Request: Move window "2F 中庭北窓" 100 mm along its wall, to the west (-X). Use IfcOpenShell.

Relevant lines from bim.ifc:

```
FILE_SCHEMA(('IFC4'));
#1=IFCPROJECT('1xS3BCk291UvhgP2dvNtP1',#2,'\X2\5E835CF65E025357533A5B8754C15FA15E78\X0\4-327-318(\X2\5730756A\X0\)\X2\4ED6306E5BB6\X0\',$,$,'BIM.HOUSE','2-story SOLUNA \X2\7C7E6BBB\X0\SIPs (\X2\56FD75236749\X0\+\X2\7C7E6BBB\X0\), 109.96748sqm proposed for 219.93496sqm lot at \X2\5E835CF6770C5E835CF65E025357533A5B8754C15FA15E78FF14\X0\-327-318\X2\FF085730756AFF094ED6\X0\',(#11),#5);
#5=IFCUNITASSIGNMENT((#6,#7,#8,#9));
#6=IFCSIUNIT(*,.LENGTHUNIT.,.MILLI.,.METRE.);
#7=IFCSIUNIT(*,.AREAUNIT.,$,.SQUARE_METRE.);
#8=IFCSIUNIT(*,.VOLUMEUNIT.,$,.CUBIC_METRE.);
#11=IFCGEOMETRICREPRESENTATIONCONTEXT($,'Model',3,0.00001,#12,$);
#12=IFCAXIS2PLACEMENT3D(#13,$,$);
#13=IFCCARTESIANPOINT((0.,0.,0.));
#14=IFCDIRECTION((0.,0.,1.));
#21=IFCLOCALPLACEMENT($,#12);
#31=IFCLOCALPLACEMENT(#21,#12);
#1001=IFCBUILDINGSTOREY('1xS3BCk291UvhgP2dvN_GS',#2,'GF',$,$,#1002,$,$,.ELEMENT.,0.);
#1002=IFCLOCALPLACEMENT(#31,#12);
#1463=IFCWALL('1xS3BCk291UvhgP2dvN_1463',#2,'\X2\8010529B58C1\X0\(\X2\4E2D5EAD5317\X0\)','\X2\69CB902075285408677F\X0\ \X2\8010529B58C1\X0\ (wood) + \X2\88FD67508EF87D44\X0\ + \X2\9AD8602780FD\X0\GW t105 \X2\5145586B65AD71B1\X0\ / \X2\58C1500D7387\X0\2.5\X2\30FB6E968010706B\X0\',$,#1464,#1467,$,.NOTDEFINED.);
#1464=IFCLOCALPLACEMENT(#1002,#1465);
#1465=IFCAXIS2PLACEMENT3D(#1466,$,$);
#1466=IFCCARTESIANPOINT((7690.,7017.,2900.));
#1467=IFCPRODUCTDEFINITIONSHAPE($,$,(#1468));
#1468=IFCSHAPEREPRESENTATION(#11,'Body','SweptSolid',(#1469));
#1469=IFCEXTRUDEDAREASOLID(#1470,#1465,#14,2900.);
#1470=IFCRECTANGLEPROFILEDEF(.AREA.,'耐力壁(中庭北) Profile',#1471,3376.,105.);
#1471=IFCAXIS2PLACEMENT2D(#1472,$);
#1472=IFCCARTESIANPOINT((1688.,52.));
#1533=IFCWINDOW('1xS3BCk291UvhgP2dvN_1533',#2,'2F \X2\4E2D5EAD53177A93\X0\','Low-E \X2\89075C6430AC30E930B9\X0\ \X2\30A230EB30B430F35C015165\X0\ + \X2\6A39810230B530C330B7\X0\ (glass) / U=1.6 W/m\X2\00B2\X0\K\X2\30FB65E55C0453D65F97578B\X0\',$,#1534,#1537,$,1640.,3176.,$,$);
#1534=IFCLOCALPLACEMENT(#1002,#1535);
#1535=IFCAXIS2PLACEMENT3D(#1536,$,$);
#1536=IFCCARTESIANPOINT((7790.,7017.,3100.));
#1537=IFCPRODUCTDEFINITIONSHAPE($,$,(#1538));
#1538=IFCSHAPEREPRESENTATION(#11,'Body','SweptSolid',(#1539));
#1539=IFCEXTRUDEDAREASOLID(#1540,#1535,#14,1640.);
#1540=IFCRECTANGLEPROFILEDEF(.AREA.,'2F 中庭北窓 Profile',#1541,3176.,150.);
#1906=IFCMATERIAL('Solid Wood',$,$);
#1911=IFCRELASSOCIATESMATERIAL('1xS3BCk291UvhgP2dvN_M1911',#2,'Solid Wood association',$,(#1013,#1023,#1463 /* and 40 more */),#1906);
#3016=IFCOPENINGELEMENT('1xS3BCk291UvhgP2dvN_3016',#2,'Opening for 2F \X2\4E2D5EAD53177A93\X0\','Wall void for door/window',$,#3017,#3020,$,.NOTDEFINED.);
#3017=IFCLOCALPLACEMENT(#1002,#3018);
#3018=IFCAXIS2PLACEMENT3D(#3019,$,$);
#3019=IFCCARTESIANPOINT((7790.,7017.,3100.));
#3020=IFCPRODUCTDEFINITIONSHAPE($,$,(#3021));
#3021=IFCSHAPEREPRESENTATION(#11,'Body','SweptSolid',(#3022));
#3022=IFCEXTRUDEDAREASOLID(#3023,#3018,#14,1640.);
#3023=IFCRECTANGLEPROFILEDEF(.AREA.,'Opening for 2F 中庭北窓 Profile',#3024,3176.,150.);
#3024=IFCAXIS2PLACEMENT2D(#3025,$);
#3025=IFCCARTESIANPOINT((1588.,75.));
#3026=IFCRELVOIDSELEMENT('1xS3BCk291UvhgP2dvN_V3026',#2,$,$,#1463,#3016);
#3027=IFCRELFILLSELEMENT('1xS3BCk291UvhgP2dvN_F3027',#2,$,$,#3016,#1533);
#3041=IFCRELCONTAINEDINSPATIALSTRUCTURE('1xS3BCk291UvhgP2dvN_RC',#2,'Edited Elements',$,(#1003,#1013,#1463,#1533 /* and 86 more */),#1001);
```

```python
import ifcopenshell
import ifcopenshell.api.geometry
import ifcopenshell.util.placement
import ifcopenshell.util.unit

model = ifcopenshell.open("bim.ifc")
unit_scale = ifcopenshell.util.unit.calculate_unit_scale(model)

window = model.by_id(1533)
opening = window.FillsVoids[0].RelatingOpeningElement
wall = opening.VoidsElements[0].RelatingBuildingElement

wall_matrix = ifcopenshell.util.placement.get_local_placement(wall.ObjectPlacement)
shift = wall_matrix[:3, 0] * -0.1 / unit_scale
before = ifcopenshell.util.placement.get_local_placement(window.ObjectPlacement)[:3, 3].copy()

# The window is not placed relative to its opening, so move both.
for product in (opening, window):
    matrix = ifcopenshell.util.placement.get_local_placement(product.ObjectPlacement)
    matrix[:3, 3] += shift
    ifcopenshell.api.geometry.edit_object_placement(model, product=product, matrix=matrix, is_si=False)

after = ifcopenshell.util.placement.get_local_placement(window.ObjectPlacement)[:3, 3]
print("window moved by", (after - before).round(3) + 0.0)

model.write("bim_v2.ifc")
```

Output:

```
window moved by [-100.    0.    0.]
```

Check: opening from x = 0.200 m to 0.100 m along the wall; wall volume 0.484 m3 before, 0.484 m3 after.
